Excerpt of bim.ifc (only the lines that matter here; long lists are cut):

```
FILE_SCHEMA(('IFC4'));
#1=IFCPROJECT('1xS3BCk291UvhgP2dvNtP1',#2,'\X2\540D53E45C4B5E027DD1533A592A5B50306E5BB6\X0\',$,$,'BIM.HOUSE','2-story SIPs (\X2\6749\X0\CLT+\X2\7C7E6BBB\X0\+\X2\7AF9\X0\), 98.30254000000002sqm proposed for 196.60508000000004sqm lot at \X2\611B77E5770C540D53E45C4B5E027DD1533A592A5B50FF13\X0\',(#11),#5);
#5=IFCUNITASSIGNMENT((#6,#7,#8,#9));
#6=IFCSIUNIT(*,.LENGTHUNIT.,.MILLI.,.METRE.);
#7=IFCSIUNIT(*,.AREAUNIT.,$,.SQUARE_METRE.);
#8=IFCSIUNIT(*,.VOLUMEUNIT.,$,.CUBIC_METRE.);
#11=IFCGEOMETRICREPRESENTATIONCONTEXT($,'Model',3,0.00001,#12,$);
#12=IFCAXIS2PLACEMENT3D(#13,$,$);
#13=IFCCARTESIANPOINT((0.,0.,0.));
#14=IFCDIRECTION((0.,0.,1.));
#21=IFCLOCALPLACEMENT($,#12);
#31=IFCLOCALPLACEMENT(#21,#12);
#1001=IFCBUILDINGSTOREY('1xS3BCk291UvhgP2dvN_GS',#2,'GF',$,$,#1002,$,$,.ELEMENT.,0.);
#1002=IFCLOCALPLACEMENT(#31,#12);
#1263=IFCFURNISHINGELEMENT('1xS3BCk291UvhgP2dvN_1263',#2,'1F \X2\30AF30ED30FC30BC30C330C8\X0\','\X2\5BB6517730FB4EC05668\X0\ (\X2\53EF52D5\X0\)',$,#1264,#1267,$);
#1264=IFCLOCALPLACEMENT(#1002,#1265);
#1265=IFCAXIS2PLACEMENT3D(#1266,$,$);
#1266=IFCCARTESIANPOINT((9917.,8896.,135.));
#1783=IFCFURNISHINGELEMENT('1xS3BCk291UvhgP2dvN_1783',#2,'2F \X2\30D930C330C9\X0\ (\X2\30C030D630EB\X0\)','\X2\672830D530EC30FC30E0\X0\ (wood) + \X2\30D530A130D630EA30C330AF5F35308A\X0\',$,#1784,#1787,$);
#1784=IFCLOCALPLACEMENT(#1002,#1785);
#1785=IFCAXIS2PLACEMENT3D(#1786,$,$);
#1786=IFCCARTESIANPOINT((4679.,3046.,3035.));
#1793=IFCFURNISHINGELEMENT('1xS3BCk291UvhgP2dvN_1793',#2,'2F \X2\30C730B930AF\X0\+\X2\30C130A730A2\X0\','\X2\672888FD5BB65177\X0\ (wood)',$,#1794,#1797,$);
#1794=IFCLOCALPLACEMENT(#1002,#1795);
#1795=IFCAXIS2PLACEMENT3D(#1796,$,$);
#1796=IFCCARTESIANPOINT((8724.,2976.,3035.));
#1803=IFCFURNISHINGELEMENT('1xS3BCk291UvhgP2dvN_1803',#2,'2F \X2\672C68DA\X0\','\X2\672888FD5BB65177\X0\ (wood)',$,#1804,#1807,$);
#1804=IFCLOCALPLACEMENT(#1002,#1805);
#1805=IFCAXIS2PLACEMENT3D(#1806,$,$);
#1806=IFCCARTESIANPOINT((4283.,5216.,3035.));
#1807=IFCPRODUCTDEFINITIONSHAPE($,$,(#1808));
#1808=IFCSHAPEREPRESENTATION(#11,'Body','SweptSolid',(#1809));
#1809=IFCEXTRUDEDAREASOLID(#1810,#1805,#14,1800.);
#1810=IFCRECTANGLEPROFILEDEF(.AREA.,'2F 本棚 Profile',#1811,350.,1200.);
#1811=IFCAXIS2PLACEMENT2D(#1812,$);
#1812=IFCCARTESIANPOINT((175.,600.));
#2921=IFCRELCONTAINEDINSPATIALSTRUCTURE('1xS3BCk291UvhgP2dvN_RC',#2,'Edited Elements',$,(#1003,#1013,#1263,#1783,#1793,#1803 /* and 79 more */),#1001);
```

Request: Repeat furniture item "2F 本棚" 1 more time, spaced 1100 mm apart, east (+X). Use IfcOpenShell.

```python
import numpy as np
import ifcopenshell
import ifcopenshell.api.geometry
import ifcopenshell.api.root
import ifcopenshell.util.element
import ifcopenshell.util.placement
import ifcopenshell.util.unit

model = ifcopenshell.open("bim.ifc")
unit_scale = ifcopenshell.util.unit.calculate_unit_scale(model)


def reuse_history(source, copy):
    """copy_class also copies each property set's owner history, people and application; keep the originals."""
    for rel in copy.IsDefinedBy:
        if rel.is_a("IfcRelDefinesByProperties") and (history := rel.RelatingPropertyDefinition.OwnerHistory):
            rel.RelatingPropertyDefinition.OwnerHistory = source.OwnerHistory
            ifcopenshell.util.element.remove_deep2(model, history)


source = model.by_id(1803)
base = ifcopenshell.util.placement.get_local_placement(source.ObjectPlacement)
step = np.array([1.0, 0.0, 0.0]) * 1.1 / unit_scale

for i in range(1, 2):
    copy = ifcopenshell.api.root.copy_class(model, product=source)
    copy.Representation = ifcopenshell.util.element.copy_deep(
        model, source.Representation, exclude=["IfcGeometricRepresentationContext", "IfcRepresentationMap"]
    )
    reuse_history(source, copy)
    matrix = base.copy()
    matrix[:3, 3] += i * step
    print("added at", matrix[:3, 3].round(3) + 0.0)
    ifcopenshell.api.geometry.edit_object_placement(model, product=copy, matrix=matrix, is_si=False)

model.write("bim-out.ifc")
```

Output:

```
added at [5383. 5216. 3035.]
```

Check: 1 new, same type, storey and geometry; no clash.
